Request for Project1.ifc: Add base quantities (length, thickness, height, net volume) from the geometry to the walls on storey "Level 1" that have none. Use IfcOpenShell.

First a look at what the model holds.

```python
import ifcopenshell
import ifcopenshell.util.element
import ifcopenshell.util.unit

model = ifcopenshell.open("Project1.ifc")
print(model.schema)
for unit_type in ("LENGTHUNIT", "AREAUNIT", "VOLUMEUNIT"):
    print(unit_type, ifcopenshell.util.unit.calculate_unit_scale(model, unit_type))
storey = next(s for s in model.by_type("IfcBuildingStorey") if s.Name == "Level 1")
walls = [e for e in ifcopenshell.util.element.get_decomposition(storey) if e.is_a("IfcWall")]
for e in sorted(walls, key=lambda e: e.id()):
    print(e.id(), e.is_a(), e.Name, list(ifcopenshell.util.element.get_psets(e, qtos_only=True)), sep=" | ")
```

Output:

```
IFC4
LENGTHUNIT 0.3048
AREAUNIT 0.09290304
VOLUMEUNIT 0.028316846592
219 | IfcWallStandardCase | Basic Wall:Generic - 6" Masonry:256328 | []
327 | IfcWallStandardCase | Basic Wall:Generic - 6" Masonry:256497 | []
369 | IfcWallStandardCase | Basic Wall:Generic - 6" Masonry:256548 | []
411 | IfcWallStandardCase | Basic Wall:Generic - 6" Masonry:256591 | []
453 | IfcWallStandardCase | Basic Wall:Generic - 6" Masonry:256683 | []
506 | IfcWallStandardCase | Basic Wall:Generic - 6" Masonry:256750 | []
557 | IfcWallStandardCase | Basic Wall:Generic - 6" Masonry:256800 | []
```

```python
import ifcopenshell
import ifcopenshell.api.pset
import ifcopenshell.geom
import ifcopenshell.util.element
import ifcopenshell.util.shape
import ifcopenshell.util.unit

model = ifcopenshell.open("Project1.ifc")
unit_scale = ifcopenshell.util.unit.calculate_unit_scale(model)
volume_scale = ifcopenshell.util.unit.calculate_unit_scale(model, "VOLUMEUNIT")
settings = ifcopenshell.geom.settings()

storey = next(s for s in model.by_type("IfcBuildingStorey") if s.Name == "Level 1")
walls = [e for e in ifcopenshell.util.element.get_decomposition(storey) if e.is_a("IfcWall")]

for e in sorted(walls, key=lambda e: e.id()):
    if ifcopenshell.util.element.get_psets(e, qtos_only=True, should_inherit=False):
        continue
    # Geometry comes back in metres, in the element's own axes.
    shape = ifcopenshell.geom.create_shape(settings, e)
    values = {
        "Length": ifcopenshell.util.shape.get_x(shape.geometry) / unit_scale,
        "Width": ifcopenshell.util.shape.get_y(shape.geometry) / unit_scale,
        "Height": ifcopenshell.util.shape.get_z(shape.geometry) / unit_scale,
        "NetVolume": ifcopenshell.util.shape.get_volume(shape.geometry) / volume_scale,
    }
    qto = ifcopenshell.api.pset.add_qto(model, product=e, name="Qto_WallBaseQuantities")
    ifcopenshell.api.pset.edit_qto(model, qto=qto, properties=values)
    print(e.id(), {k: round(v, 3) for k, v in values.items()})

model.write("Project1_rev.ifc")
```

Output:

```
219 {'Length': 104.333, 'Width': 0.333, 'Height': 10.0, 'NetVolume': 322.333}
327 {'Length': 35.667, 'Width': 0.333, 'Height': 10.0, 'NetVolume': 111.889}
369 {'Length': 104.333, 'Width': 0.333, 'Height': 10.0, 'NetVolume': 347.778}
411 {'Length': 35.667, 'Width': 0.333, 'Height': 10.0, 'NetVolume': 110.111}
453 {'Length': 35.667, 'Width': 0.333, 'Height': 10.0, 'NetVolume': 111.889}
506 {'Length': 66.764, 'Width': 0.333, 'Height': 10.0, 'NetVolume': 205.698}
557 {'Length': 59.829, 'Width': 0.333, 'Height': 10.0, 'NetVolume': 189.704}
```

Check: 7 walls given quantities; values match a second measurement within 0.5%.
